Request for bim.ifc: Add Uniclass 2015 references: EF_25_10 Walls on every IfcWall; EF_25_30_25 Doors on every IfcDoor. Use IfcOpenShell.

First a look at what the model holds.

```python
import ifcopenshell

model = ifcopenshell.open("bim.ifc")
print(model.schema)
print("classifications:", [c.Name for c in model.by_type("IfcClassification")])
for ifc_class in ("IfcDoor", "IfcRoof", "IfcStair", "IfcWall", "IfcWindow"):
    print(ifc_class, len(model.by_type(ifc_class)))
```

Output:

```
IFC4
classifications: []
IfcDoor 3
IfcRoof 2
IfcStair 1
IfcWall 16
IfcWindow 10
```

```python
import ifcopenshell
import ifcopenshell.api.classification

model = ifcopenshell.open("bim.ifc")

system = ifcopenshell.api.classification.add_classification(model, classification="Uniclass 2015")

codes = {
    "IfcWall": ("EF_25_10", "Walls"),
    "IfcDoor": ("EF_25_30_25", "Doors"),
}
for ifc_class, (code, name) in codes.items():
    products = model.by_type(ifc_class)
    ifcopenshell.api.classification.add_reference(
        model, products=products, classification=system, identification=code, name=name
    )
    print(code, len(products))

model.write("bim_v2.ifc")
```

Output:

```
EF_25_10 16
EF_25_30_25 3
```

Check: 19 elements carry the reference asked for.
